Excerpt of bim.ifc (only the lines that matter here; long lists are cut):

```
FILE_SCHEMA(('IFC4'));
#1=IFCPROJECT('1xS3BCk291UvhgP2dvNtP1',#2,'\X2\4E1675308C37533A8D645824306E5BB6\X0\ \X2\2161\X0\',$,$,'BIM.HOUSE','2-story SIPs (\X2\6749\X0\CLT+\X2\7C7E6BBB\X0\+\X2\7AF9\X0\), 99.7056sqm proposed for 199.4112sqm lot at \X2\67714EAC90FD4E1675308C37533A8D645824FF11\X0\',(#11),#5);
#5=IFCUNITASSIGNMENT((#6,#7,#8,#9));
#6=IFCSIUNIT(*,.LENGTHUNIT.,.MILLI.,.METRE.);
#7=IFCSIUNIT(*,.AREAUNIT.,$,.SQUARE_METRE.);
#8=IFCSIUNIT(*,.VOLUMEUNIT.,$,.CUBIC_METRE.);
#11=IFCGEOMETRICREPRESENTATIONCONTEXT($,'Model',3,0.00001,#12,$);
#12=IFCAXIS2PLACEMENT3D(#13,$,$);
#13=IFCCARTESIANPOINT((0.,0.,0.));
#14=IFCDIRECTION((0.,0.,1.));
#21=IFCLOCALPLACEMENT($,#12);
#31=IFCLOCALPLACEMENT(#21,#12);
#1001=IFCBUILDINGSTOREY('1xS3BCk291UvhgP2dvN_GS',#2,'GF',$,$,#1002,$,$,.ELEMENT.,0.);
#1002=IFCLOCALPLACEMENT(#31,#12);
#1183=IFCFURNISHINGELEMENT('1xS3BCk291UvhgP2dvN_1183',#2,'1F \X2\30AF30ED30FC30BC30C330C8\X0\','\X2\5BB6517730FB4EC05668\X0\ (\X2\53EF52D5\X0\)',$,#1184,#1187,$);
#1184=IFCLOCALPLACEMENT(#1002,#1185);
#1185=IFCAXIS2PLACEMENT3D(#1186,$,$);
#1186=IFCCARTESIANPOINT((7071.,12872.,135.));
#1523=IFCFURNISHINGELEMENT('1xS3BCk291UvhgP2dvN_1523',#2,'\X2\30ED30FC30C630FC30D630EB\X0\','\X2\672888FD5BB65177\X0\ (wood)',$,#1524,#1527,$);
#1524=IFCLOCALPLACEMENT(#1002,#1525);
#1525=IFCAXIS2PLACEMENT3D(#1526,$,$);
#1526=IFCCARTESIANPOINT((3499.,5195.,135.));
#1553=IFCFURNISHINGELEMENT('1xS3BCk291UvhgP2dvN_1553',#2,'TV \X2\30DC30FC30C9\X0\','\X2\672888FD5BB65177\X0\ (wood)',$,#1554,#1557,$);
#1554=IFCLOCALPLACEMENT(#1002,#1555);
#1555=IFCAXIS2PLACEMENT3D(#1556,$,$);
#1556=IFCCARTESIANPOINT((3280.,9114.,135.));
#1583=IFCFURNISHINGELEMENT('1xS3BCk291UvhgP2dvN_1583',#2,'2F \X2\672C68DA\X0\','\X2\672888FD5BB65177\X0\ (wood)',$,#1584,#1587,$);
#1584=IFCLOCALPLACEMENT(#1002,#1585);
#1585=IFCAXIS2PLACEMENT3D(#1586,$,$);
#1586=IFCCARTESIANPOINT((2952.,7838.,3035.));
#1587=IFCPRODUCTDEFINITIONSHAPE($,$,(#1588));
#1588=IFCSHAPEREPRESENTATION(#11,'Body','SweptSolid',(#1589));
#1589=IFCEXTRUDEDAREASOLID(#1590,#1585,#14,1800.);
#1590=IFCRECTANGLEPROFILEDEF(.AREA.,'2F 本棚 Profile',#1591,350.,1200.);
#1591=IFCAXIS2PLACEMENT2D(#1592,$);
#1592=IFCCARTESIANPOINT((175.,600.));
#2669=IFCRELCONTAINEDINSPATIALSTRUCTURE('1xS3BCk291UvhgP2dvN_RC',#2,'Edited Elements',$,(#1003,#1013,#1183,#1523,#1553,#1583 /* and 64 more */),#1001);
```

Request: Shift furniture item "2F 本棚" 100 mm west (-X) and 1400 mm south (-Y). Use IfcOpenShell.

```python
import ifcopenshell
import ifcopenshell.api.geometry
import ifcopenshell.util.placement

model = ifcopenshell.open("bim.ifc")

item = model.by_guid("1xS3BCk291UvhgP2dvN_1583")
matrix = ifcopenshell.util.placement.get_local_placement(item.ObjectPlacement)
matrix[0, 3] -= 100.0
matrix[1, 3] -= 1400.0
ifcopenshell.api.geometry.edit_object_placement(model, product=item, matrix=matrix, is_si=False)

print(ifcopenshell.util.placement.get_local_placement(item.ObjectPlacement).round(3) + 0.0)

model.write("bim-out.ifc")
```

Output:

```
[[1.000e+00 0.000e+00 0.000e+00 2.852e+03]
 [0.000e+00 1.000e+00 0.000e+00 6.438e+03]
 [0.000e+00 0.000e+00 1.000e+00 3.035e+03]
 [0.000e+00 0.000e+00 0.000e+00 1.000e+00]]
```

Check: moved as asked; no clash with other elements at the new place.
